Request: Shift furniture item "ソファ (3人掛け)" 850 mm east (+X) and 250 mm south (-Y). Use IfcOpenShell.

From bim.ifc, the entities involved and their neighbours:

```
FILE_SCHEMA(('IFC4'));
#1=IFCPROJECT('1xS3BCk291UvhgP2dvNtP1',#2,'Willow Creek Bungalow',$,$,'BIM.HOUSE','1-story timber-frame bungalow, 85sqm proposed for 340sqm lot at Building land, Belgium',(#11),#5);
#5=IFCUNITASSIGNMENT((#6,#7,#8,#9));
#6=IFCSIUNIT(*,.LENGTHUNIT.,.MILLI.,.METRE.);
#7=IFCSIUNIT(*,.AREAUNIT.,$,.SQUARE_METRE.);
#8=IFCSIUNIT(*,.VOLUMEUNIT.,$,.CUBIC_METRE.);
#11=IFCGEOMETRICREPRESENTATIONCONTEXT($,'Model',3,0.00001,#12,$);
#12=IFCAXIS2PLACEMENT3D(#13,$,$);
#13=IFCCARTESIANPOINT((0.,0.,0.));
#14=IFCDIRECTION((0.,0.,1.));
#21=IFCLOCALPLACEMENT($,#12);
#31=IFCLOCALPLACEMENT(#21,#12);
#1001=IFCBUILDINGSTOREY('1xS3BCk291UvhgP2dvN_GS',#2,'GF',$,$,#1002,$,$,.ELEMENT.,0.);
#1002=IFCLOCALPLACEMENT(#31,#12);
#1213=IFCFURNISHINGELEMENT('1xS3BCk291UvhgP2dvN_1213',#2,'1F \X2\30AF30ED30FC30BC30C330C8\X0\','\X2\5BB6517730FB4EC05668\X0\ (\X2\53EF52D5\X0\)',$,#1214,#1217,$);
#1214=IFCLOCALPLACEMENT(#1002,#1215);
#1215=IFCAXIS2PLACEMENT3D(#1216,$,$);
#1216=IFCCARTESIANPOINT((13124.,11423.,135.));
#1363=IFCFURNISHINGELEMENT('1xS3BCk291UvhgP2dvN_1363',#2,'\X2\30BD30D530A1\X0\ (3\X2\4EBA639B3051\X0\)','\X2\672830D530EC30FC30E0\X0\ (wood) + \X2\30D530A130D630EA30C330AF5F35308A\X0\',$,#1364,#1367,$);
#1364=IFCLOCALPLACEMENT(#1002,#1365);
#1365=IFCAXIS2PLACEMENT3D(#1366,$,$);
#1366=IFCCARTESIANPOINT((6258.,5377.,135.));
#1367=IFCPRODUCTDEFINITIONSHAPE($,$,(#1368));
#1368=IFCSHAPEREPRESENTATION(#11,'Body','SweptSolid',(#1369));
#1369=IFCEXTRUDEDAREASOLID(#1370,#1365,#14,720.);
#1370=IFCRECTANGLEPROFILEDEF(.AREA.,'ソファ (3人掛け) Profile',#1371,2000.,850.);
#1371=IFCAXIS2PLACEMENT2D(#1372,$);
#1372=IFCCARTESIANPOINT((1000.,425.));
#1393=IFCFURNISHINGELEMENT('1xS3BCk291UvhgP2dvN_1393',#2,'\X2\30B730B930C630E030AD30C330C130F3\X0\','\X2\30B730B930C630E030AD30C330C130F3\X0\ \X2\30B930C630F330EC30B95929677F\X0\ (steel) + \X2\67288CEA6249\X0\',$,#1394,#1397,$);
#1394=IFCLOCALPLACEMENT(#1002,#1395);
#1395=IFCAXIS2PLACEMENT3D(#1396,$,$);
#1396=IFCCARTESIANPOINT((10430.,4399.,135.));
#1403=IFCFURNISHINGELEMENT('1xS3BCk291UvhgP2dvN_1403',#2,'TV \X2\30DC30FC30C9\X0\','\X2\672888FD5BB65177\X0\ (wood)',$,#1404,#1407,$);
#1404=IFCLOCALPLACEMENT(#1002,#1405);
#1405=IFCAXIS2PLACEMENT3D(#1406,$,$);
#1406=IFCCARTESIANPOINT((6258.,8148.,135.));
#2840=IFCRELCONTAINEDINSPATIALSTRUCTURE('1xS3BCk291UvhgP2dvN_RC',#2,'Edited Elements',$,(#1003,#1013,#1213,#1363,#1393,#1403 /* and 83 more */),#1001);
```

```python
import ifcopenshell
import ifcopenshell.api.geometry
import ifcopenshell.util.placement
import ifcopenshell.util.unit

model = ifcopenshell.open("bim.ifc")
unit_scale = ifcopenshell.util.unit.calculate_unit_scale(model)

item = model.by_id(1363)
matrix = ifcopenshell.util.placement.get_local_placement(item.ObjectPlacement)
matrix[0, 3] += 0.85 / unit_scale
matrix[1, 3] -= 0.25 / unit_scale
ifcopenshell.api.geometry.edit_object_placement(model, product=item, matrix=matrix, is_si=False)

print(ifcopenshell.util.placement.get_local_placement(item.ObjectPlacement).round(3) + 0.0)

model.write("bim_updated.ifc")
```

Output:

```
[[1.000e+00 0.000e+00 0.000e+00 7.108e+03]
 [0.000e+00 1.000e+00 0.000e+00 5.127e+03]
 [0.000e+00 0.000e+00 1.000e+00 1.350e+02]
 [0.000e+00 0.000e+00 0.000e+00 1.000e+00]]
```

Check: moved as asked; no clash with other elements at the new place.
